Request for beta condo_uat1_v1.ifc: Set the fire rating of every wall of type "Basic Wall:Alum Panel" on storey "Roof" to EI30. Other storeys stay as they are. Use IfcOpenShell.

First a look at what the model holds.

```python
import ifcopenshell
import ifcopenshell.util.element

model = ifcopenshell.open("beta condo_uat1_v1.ifc")
print(model.schema)
storey = next(s for s in model.by_type("IfcBuildingStorey") if s.Name == "Roof")
walls = [e for e in ifcopenshell.util.element.get_decomposition(storey) if e.is_a("IfcWall")]
seen = {}
for e in walls:
    element_type = ifcopenshell.util.element.get_type(e)
    key = (element_type.Name if element_type != e and element_type else None, ifcopenshell.util.element.get_pset(e, "Pset_WallCommon", "FireRating"))
    seen[key] = seen.get(key, 0) + 1
for (name, value), count in sorted(seen.items(), key=str):
    print(count, "x", name, "|", value)
```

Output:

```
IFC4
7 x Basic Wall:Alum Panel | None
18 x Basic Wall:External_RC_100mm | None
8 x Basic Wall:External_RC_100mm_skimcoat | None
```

```python
import ifcopenshell
import ifcopenshell.api.pset
import ifcopenshell.util.element

model = ifcopenshell.open("beta condo_uat1_v1.ifc")

storey = next(s for s in model.by_type("IfcBuildingStorey") if s.Name == "Roof")
walls = [e for e in ifcopenshell.util.element.get_decomposition(storey) if e.is_a("IfcWall")]

count = 0
for e in walls:
    element_type = ifcopenshell.util.element.get_type(e)
    if element_type in (None, e) or element_type.Name != "Basic Wall:Alum Panel":
        continue
    # add_pset returns the element's existing set when there is one.
    pset = ifcopenshell.api.pset.add_pset(model, product=e, name="Pset_WallCommon")
    ifcopenshell.api.pset.edit_pset(model, pset=pset, properties={"FireRating": "EI30"})
    count += 1

print(count, "walls updated")

model.write("beta condo_uat1_v1-out.ifc")
```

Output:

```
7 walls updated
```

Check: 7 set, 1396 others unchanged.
